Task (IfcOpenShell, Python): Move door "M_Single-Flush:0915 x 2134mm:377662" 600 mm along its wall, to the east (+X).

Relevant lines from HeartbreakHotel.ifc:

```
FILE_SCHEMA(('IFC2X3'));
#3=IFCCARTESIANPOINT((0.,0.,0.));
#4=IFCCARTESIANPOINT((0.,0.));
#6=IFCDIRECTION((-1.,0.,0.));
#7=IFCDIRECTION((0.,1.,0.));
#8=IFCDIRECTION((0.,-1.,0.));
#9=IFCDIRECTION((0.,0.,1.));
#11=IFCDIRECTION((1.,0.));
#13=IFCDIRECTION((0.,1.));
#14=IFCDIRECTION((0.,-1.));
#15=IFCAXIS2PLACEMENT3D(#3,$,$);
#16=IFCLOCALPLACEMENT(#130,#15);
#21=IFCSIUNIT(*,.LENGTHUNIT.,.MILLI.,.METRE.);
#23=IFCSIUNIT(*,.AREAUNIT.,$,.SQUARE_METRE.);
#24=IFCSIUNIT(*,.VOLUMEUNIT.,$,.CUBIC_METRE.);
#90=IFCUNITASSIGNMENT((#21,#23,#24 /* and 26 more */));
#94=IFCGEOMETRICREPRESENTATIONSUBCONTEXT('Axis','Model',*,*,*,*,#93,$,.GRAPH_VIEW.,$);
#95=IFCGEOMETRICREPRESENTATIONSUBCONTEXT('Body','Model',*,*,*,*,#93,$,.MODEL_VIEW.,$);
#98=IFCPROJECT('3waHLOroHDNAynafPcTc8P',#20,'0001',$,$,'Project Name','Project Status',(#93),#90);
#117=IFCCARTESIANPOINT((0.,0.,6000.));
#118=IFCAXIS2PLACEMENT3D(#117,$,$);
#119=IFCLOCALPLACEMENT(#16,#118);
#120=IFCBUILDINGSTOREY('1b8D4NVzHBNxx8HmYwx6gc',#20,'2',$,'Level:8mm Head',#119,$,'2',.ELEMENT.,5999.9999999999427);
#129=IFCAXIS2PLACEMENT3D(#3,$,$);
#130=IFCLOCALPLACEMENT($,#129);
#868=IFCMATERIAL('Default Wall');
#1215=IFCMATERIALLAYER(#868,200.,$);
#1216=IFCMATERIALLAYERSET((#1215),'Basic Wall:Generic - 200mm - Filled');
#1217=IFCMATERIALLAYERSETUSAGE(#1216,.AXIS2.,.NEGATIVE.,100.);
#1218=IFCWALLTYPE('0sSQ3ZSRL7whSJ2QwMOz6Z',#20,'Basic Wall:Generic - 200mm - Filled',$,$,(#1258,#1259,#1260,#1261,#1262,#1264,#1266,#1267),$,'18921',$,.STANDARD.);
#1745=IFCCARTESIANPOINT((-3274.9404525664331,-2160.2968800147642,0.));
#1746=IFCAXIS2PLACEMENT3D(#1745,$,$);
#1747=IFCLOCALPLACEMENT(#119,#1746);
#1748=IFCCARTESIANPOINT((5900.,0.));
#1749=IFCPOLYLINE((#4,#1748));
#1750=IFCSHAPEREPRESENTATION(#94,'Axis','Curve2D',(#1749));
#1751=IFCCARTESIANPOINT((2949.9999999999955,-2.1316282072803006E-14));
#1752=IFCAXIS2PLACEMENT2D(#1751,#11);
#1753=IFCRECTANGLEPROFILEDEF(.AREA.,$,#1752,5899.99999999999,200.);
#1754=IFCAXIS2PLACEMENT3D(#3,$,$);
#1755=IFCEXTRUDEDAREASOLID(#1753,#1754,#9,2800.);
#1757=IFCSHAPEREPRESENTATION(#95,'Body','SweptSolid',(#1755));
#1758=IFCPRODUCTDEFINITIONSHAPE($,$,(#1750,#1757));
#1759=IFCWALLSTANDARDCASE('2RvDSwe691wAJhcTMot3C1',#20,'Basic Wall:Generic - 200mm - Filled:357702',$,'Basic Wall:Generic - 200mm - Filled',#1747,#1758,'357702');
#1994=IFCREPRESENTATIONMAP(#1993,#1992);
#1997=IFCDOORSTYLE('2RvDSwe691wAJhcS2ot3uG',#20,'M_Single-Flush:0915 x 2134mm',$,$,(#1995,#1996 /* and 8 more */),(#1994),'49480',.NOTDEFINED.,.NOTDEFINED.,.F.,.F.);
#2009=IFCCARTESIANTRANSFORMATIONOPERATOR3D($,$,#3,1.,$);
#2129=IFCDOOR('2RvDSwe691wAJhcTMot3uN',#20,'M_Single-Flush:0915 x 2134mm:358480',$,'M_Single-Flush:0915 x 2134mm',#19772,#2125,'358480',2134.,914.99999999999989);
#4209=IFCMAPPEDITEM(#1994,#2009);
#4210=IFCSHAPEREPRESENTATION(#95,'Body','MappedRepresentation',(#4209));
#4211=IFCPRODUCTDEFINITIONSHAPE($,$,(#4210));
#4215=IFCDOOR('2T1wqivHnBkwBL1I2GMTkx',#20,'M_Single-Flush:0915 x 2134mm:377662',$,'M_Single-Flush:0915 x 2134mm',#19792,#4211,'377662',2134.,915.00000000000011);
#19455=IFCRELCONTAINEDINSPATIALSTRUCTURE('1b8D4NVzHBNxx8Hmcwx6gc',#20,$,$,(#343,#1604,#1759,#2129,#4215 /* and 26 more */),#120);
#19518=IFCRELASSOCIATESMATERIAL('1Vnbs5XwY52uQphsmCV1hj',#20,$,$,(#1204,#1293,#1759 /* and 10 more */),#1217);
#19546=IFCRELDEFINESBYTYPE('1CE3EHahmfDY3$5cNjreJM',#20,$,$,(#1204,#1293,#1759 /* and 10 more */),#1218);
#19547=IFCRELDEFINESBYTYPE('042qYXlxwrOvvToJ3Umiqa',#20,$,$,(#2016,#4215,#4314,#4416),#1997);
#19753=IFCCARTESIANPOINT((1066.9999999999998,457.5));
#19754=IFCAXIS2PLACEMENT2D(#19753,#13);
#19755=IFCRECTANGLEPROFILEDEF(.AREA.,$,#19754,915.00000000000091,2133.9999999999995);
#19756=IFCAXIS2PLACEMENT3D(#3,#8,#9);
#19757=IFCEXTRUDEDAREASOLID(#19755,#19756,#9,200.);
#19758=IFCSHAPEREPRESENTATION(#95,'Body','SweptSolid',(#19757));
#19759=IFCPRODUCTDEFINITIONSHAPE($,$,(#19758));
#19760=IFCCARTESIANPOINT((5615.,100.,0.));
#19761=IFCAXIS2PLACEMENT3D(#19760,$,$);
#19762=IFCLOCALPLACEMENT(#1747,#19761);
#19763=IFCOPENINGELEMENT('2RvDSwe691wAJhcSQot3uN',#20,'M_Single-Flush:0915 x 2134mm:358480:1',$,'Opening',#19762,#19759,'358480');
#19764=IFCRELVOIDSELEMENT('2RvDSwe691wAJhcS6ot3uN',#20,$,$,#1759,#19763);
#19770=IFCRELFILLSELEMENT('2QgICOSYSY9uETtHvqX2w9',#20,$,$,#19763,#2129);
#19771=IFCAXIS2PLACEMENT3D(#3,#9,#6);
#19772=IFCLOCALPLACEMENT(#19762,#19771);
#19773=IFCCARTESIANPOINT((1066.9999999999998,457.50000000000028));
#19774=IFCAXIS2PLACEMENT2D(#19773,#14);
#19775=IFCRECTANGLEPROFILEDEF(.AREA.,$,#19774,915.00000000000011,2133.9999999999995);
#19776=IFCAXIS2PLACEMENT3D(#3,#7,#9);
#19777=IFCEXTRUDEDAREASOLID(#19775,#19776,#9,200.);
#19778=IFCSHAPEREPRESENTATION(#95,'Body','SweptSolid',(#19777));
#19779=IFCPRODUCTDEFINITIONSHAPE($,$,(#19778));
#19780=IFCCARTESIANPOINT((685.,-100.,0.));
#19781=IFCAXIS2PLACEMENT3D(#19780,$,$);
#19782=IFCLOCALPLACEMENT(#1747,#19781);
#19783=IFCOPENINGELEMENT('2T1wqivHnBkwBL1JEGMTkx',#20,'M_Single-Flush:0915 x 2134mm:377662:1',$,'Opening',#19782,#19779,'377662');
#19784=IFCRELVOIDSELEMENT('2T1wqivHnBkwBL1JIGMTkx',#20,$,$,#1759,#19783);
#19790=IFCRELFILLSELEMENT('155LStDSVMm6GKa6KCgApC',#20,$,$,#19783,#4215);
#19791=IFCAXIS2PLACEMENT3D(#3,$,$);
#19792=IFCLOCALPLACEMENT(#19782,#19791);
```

```python
import ifcopenshell
import ifcopenshell.api.geometry
import ifcopenshell.util.placement

model = ifcopenshell.open("HeartbreakHotel.ifc")

door = model.by_guid("2T1wqivHnBkwBL1I2GMTkx")
opening = door.FillsVoids[0].RelatingOpeningElement
wall = opening.VoidsElements[0].RelatingBuildingElement

wall_matrix = ifcopenshell.util.placement.get_local_placement(wall.ObjectPlacement)
shift = wall_matrix[:3, 0] * 600.0
before = ifcopenshell.util.placement.get_local_placement(door.ObjectPlacement)[:3, 3].copy()

# The door is placed relative to its opening, so it follows when the opening moves.
matrix = ifcopenshell.util.placement.get_local_placement(opening.ObjectPlacement)
matrix[:3, 3] += shift
ifcopenshell.api.geometry.edit_object_placement(
    model, product=opening, matrix=matrix, is_si=False, should_transform_children=True
)

after = ifcopenshell.util.placement.get_local_placement(door.ObjectPlacement)[:3, 3]
print("door moved by", (after - before).round(3) + 0.0)

model.write("HeartbreakHotel_v2.ifc")
```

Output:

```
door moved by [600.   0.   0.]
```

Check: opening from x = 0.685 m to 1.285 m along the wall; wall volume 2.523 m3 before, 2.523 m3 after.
